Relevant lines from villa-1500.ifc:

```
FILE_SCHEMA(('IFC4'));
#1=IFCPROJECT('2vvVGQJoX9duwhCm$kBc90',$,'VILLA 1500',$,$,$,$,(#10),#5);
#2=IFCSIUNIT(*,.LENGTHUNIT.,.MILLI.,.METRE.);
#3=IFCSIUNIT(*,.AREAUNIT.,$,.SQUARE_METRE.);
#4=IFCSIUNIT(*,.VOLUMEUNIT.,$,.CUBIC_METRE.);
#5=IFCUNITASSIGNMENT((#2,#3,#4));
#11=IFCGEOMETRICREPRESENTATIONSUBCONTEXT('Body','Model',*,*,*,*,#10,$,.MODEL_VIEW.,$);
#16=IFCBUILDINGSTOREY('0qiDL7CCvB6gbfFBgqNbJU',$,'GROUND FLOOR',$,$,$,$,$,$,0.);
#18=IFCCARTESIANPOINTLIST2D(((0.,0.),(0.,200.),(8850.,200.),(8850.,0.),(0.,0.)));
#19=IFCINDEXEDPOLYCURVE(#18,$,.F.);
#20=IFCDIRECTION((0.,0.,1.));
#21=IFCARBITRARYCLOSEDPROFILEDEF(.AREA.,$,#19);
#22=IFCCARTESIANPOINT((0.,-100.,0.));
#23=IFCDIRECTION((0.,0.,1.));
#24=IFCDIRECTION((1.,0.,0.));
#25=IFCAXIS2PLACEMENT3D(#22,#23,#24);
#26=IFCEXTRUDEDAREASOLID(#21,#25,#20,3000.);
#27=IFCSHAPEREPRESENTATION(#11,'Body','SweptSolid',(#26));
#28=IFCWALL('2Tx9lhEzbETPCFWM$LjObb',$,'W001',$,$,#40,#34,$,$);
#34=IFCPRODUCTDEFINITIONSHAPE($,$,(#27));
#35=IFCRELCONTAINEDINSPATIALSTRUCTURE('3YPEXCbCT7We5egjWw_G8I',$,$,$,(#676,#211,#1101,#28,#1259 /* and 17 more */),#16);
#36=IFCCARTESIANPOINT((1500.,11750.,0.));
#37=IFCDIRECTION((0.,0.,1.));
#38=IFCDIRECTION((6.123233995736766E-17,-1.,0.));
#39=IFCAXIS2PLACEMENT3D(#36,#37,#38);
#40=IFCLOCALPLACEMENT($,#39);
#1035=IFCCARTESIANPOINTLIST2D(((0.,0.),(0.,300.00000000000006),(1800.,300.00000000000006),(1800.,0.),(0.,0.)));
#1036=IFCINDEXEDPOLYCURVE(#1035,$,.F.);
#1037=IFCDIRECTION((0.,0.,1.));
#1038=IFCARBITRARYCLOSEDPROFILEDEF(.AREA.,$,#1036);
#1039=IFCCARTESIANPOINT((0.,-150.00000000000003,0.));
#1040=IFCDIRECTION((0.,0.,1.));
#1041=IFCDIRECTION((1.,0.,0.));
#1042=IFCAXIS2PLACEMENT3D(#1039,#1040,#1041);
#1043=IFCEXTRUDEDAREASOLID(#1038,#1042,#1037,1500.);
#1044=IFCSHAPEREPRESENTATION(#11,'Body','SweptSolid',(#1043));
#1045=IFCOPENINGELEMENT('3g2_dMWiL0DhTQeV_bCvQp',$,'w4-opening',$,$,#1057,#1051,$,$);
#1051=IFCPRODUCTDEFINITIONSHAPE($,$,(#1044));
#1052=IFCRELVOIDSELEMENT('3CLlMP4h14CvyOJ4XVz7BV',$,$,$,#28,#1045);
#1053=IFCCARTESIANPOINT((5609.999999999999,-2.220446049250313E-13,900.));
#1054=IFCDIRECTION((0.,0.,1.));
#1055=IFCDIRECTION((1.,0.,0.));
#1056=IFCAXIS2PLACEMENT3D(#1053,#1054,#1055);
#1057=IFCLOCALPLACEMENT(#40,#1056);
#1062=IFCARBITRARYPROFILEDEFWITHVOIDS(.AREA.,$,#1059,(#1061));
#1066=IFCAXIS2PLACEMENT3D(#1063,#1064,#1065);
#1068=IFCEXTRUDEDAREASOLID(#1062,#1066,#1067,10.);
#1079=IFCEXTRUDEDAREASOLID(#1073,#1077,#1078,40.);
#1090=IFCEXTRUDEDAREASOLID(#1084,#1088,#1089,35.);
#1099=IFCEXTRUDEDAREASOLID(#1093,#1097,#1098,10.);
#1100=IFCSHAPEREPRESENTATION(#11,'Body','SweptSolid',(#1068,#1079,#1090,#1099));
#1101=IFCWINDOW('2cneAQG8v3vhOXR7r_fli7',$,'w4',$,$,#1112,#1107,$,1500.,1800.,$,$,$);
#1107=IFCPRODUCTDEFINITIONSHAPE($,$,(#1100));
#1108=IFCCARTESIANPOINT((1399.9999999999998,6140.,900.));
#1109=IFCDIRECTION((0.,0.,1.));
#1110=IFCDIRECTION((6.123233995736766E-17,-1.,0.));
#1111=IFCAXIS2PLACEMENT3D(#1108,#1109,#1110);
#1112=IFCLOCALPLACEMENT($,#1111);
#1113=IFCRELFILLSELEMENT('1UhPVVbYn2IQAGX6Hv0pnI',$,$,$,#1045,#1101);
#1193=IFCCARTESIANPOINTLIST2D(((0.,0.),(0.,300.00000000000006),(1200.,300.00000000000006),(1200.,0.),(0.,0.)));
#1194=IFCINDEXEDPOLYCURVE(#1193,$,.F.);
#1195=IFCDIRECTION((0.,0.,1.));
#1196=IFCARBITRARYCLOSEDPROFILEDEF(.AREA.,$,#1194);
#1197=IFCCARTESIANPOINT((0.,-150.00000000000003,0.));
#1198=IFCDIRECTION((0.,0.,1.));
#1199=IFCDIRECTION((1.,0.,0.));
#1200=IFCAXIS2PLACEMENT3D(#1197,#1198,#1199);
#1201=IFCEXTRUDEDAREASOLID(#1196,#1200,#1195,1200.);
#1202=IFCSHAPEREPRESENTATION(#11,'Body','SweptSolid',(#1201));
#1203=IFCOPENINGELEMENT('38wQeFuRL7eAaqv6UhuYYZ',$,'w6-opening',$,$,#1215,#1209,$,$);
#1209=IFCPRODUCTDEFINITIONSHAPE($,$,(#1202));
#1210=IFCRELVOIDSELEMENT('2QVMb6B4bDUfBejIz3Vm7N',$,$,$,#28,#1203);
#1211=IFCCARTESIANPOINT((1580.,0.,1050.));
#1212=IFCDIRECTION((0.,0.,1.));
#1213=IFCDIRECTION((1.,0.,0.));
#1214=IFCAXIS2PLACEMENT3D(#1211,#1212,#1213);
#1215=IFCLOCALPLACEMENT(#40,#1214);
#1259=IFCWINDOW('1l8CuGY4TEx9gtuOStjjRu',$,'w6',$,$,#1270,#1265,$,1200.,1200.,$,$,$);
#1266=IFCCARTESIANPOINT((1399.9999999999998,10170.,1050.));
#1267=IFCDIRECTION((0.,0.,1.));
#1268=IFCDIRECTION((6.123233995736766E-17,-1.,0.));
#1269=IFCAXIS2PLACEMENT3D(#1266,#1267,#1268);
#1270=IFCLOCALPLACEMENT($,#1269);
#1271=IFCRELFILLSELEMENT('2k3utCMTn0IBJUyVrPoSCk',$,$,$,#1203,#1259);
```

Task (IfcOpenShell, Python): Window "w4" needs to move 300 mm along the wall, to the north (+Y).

```python
import ifcopenshell
import ifcopenshell.api.geometry
import ifcopenshell.util.placement

model = ifcopenshell.open("villa-1500.ifc")

window = model.by_id(1101)
opening = window.FillsVoids[0].RelatingOpeningElement
wall = opening.VoidsElements[0].RelatingBuildingElement

wall_matrix = ifcopenshell.util.placement.get_local_placement(wall.ObjectPlacement)
shift = wall_matrix[:3, 0] * -300.0
before = ifcopenshell.util.placement.get_local_placement(window.ObjectPlacement)[:3, 3].copy()

# The window is not placed relative to its opening, so move both.
for product in (opening, window):
    matrix = ifcopenshell.util.placement.get_local_placement(product.ObjectPlacement)
    matrix[:3, 3] += shift
    ifcopenshell.api.geometry.edit_object_placement(model, product=product, matrix=matrix, is_si=False)

after = ifcopenshell.util.placement.get_local_placement(window.ObjectPlacement)[:3, 3]
print("window moved by", (after - before).round(3) + 0.0)

model.write("villa-1500_rev.ifc")
```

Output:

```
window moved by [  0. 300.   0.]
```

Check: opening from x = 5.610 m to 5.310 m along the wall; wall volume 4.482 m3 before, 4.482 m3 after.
